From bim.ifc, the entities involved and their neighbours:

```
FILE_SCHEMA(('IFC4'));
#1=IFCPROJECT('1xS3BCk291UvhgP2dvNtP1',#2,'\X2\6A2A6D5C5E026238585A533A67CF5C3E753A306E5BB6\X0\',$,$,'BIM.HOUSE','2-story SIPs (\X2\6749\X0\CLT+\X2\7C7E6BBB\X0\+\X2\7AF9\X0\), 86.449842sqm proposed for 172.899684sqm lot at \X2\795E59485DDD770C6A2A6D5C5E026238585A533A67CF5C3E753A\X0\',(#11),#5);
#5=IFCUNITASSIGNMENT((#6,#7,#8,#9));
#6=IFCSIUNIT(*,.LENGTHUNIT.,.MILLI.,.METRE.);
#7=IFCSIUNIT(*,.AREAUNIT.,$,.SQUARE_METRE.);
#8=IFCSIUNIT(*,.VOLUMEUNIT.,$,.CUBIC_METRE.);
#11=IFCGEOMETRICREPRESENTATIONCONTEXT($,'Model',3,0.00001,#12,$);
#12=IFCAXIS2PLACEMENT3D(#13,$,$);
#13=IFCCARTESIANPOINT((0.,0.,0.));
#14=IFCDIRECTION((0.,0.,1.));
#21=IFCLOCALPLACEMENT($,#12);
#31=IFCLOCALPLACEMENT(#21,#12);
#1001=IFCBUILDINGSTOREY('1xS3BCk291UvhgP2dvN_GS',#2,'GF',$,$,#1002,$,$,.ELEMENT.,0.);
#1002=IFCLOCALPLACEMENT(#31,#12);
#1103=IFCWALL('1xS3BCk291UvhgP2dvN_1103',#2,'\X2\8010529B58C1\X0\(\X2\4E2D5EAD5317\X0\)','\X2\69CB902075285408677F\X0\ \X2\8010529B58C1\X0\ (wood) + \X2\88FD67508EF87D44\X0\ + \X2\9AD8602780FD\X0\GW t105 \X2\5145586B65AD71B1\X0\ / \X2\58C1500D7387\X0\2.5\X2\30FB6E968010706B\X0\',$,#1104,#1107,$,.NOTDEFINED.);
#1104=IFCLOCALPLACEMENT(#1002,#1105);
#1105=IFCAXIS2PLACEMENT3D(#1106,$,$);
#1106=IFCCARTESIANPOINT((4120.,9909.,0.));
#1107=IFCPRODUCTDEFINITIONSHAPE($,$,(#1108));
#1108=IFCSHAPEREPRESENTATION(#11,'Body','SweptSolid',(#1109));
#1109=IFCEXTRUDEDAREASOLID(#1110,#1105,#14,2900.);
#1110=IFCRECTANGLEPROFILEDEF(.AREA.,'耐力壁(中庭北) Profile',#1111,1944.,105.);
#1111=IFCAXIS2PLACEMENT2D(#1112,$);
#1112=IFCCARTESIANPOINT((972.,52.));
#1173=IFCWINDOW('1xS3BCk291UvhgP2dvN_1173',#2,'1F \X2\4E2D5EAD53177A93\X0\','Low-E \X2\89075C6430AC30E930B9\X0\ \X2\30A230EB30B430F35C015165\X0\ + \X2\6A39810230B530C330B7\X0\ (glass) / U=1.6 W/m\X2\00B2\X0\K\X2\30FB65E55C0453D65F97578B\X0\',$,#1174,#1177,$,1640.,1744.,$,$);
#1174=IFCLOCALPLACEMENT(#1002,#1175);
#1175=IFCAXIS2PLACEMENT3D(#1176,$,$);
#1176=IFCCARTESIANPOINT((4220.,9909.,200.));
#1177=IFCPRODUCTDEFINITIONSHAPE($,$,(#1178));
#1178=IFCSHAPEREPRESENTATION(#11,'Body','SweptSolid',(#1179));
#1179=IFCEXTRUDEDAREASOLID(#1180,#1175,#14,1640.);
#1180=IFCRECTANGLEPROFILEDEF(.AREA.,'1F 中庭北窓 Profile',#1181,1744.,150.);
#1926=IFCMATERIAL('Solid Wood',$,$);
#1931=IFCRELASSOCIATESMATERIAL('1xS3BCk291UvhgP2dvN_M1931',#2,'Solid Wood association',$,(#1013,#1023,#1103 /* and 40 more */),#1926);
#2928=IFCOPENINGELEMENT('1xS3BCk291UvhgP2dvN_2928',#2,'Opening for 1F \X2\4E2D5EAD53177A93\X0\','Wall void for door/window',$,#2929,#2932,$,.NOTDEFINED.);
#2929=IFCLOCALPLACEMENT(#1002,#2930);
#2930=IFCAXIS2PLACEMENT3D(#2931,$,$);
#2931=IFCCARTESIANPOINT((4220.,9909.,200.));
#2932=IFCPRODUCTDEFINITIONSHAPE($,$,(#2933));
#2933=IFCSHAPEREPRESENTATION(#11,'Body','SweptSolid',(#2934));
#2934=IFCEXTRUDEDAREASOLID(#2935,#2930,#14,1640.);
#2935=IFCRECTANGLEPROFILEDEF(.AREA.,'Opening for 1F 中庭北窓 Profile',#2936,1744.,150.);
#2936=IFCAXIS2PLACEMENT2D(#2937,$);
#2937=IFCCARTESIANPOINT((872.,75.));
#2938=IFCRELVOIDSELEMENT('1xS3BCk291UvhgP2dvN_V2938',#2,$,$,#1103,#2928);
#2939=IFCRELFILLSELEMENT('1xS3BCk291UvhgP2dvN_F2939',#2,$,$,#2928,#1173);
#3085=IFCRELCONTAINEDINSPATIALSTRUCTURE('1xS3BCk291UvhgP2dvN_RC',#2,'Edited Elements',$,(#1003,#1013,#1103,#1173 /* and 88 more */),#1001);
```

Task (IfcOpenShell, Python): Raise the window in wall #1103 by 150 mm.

```python
import numpy as np
import ifcopenshell
import ifcopenshell.api.geometry
import ifcopenshell.util.placement
import ifcopenshell.util.unit

model = ifcopenshell.open("bim.ifc")
unit_scale = ifcopenshell.util.unit.calculate_unit_scale(model)

window = model.by_id(1173)
opening = window.FillsVoids[0].RelatingOpeningElement
dz = 0.15 / unit_scale

shift = np.array([0.0, 0.0, dz])
# The window is not placed relative to its opening, so move both.
for product in (opening, window):
    matrix = ifcopenshell.util.placement.get_local_placement(product.ObjectPlacement)
    matrix[:3, 3] += shift
    ifcopenshell.api.geometry.edit_object_placement(model, product=product, matrix=matrix, is_si=False)

print(f"moved by {dz * unit_scale:+.3f} m")

model.write("bim_edited.ifc")
```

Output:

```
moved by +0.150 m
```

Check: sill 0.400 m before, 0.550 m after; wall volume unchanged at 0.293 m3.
